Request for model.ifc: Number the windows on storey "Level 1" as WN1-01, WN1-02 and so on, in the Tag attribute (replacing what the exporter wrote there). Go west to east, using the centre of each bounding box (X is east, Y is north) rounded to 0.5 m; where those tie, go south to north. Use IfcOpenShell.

First a look at what the model holds.

```python
import ifcopenshell
import ifcopenshell.util.element
import ifcopenshell.util.placement

model = ifcopenshell.open("model.ifc")
print(model.schema)
storey = next(s for s in model.by_type("IfcBuildingStorey") if s.Name == "Level 1")
windows = [e for e in ifcopenshell.util.element.get_decomposition(storey) if e.is_a("IfcWindow")]
for e in sorted(windows, key=lambda e: e.id()):
    origin = ifcopenshell.util.placement.get_local_placement(e.ObjectPlacement)[:3, 3]
    print(e.id(), e.Tag, e.Name, origin.round(2) + 0.0, sep=" | ")
```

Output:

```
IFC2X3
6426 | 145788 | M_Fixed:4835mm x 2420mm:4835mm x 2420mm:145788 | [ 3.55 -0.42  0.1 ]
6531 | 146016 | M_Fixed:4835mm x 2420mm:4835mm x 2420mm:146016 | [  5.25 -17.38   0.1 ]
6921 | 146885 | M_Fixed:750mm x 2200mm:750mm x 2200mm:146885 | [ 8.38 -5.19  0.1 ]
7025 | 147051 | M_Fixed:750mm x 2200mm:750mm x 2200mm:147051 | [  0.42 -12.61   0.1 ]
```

```python
import ifcopenshell
import ifcopenshell.geom
import ifcopenshell.util.element
import ifcopenshell.util.shape

model = ifcopenshell.open("model.ifc")
settings = ifcopenshell.geom.settings()
settings.set("use-world-coords", True)


def centre(element):
    shape = ifcopenshell.geom.create_shape(settings, element)
    return ifcopenshell.util.shape.get_bbox_centroid(shape.geometry)


storey = next(s for s in model.by_type("IfcBuildingStorey") if s.Name == "Level 1")
windows = [e for e in ifcopenshell.util.element.get_decomposition(storey) if e.is_a("IfcWindow")]

# Insertion points can sit at a corner or the storey origin, so sort by the geometry (in metres).
centres = {e: centre(e) for e in windows}
windows.sort(key=lambda e: (round(centres[e][0] / 0.5), centres[e][1]))

for i, e in enumerate(windows, start=1):
    number = f"WN1-{i:02d}"
    e.Tag = number
    print(e.id(), number)

model.write("model_v2.ifc")
```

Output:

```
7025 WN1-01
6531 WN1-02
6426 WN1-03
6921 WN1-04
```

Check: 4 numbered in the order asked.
